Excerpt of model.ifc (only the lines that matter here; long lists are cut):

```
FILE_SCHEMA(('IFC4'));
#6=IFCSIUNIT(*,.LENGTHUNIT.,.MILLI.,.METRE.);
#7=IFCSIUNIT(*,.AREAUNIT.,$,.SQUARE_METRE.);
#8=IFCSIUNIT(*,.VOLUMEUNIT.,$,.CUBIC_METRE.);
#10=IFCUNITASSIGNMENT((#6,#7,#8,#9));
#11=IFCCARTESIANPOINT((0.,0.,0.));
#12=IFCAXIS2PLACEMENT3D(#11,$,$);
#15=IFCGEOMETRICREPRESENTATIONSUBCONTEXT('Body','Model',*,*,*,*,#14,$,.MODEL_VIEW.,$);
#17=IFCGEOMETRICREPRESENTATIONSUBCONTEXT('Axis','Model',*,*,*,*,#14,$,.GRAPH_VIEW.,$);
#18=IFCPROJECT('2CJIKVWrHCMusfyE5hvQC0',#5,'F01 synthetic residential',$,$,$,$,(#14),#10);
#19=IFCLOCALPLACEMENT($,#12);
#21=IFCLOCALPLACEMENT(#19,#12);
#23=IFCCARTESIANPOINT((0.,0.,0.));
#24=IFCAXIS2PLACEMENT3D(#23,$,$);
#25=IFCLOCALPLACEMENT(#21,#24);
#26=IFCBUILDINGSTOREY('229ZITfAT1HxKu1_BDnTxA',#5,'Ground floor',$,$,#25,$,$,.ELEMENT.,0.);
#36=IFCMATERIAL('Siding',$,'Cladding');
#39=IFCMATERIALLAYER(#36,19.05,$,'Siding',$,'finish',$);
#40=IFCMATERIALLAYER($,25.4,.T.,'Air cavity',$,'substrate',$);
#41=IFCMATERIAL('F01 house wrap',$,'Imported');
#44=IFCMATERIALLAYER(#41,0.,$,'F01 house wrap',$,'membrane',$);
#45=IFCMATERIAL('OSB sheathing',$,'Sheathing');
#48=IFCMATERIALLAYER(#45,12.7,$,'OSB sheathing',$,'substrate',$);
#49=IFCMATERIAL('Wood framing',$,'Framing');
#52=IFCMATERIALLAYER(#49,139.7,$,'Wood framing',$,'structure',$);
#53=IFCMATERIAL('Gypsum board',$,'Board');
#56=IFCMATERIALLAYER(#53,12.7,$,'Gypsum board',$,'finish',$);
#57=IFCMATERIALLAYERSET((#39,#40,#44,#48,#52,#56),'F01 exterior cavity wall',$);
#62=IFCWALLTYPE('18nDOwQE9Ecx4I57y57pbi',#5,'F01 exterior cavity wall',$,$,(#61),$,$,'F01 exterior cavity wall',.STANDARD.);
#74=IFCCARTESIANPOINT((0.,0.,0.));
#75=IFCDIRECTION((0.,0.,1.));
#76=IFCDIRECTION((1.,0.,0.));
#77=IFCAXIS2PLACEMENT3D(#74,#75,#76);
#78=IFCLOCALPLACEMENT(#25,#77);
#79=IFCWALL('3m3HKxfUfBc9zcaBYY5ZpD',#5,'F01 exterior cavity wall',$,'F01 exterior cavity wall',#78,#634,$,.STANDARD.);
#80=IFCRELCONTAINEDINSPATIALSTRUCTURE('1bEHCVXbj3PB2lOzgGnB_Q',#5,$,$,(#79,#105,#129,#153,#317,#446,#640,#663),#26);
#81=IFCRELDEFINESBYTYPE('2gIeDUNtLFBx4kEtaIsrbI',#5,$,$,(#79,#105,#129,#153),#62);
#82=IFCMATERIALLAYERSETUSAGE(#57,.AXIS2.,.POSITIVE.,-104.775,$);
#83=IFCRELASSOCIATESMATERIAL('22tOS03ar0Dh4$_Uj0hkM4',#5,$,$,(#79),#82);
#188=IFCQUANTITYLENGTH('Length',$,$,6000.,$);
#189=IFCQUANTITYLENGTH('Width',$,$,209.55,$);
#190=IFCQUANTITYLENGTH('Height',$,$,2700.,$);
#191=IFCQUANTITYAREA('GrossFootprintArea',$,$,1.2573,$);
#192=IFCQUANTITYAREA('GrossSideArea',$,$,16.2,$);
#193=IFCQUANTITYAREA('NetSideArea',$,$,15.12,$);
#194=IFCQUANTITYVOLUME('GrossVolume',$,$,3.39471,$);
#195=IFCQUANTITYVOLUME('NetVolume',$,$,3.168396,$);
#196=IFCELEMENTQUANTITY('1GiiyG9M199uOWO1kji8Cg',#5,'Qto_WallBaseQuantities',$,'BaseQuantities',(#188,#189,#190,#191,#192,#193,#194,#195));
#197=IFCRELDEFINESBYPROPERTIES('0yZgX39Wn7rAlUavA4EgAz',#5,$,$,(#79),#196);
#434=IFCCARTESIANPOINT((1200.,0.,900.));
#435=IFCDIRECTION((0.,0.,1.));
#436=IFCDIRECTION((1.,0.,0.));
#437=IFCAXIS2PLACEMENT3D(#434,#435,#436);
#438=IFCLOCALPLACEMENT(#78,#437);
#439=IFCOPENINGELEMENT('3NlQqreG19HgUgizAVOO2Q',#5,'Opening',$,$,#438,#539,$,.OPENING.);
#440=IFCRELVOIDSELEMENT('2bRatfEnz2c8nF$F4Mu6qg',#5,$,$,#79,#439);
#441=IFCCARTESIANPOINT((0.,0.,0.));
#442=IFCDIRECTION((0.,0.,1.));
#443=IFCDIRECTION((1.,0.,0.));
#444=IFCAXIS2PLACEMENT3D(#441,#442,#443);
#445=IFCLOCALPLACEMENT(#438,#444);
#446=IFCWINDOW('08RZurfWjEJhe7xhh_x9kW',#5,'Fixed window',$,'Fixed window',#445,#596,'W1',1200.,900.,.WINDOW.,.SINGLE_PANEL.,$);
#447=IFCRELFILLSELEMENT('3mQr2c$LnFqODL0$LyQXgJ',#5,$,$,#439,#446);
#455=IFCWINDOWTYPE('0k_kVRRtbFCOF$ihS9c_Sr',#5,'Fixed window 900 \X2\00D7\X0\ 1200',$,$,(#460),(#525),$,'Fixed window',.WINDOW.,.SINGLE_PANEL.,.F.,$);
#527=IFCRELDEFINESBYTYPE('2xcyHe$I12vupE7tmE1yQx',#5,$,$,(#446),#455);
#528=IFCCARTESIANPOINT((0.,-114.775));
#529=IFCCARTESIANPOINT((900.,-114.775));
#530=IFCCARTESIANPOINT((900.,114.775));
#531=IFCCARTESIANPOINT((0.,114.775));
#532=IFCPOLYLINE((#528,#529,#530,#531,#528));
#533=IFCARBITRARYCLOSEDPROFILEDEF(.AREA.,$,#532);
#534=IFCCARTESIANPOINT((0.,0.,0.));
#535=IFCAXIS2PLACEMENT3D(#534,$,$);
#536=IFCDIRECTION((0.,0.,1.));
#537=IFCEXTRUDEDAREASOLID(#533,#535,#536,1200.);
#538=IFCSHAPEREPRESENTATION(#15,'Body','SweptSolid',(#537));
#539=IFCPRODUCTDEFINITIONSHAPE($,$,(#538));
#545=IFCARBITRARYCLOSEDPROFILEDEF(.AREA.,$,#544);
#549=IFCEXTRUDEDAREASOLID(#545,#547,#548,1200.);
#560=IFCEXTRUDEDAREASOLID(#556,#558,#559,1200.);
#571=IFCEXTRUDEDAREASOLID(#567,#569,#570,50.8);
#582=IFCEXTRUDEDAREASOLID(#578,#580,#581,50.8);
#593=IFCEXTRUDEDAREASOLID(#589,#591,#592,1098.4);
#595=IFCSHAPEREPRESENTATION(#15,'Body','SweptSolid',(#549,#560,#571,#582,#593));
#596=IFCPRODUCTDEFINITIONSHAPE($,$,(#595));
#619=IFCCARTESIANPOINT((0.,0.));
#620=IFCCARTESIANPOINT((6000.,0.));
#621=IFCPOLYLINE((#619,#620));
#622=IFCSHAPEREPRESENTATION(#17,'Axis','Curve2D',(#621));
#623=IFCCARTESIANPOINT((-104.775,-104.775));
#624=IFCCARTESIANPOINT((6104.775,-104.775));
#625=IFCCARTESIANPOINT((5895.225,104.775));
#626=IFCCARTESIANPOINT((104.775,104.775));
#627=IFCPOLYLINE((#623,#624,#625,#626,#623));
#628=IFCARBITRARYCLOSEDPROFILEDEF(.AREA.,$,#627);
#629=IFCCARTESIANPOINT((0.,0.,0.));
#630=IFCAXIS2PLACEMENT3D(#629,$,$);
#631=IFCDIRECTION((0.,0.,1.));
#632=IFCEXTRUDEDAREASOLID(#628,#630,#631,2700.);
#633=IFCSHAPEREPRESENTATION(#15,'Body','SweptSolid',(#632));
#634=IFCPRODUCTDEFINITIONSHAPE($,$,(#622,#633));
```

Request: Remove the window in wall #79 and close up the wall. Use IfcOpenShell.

```python
import ifcopenshell
import ifcopenshell.api.feature
import ifcopenshell.api.pset
import ifcopenshell.api.root
import ifcopenshell.geom
import ifcopenshell.util.element
import ifcopenshell.util.shape
import ifcopenshell.util.unit

model = ifcopenshell.open("model.ifc")
area_scale = ifcopenshell.util.unit.calculate_unit_scale(model, "AREAUNIT")
volume_scale = ifcopenshell.util.unit.calculate_unit_scale(model, "VOLUMEUNIT")
settings = ifcopenshell.geom.settings()


def volume(element):
    """Net volume in cubic metres, openings subtracted."""
    shape = ifcopenshell.geom.create_shape(settings, element)
    return ifcopenshell.util.shape.get_volume(shape.geometry)


window = model.by_id(446)
opening = window.FillsVoids[0].RelatingOpeningElement
wall = opening.VoidsElements[0].RelatingBuildingElement
before = volume(wall)

ifcopenshell.api.root.remove_product(model, product=window)
ifcopenshell.api.feature.remove_feature(model, feature=opening)

after = volume(wall)
thickness = 0.2096  # wall thickness in metres

# Update the wall's stored quantities.
qto = model.by_id(ifcopenshell.util.element.get_pset(wall, "Qto_WallBaseQuantities", should_inherit=False)["id"])
ifcopenshell.api.pset.edit_qto(model, qto=qto, properties={
    "NetSideArea": after / thickness / area_scale,
    "NetVolume": after / volume_scale,
})

print(f"wall volume {before:.3f} -> {after:.3f} m3")

model.write("model_rev.ifc")
```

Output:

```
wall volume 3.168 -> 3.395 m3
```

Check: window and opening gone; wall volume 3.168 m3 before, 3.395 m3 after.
